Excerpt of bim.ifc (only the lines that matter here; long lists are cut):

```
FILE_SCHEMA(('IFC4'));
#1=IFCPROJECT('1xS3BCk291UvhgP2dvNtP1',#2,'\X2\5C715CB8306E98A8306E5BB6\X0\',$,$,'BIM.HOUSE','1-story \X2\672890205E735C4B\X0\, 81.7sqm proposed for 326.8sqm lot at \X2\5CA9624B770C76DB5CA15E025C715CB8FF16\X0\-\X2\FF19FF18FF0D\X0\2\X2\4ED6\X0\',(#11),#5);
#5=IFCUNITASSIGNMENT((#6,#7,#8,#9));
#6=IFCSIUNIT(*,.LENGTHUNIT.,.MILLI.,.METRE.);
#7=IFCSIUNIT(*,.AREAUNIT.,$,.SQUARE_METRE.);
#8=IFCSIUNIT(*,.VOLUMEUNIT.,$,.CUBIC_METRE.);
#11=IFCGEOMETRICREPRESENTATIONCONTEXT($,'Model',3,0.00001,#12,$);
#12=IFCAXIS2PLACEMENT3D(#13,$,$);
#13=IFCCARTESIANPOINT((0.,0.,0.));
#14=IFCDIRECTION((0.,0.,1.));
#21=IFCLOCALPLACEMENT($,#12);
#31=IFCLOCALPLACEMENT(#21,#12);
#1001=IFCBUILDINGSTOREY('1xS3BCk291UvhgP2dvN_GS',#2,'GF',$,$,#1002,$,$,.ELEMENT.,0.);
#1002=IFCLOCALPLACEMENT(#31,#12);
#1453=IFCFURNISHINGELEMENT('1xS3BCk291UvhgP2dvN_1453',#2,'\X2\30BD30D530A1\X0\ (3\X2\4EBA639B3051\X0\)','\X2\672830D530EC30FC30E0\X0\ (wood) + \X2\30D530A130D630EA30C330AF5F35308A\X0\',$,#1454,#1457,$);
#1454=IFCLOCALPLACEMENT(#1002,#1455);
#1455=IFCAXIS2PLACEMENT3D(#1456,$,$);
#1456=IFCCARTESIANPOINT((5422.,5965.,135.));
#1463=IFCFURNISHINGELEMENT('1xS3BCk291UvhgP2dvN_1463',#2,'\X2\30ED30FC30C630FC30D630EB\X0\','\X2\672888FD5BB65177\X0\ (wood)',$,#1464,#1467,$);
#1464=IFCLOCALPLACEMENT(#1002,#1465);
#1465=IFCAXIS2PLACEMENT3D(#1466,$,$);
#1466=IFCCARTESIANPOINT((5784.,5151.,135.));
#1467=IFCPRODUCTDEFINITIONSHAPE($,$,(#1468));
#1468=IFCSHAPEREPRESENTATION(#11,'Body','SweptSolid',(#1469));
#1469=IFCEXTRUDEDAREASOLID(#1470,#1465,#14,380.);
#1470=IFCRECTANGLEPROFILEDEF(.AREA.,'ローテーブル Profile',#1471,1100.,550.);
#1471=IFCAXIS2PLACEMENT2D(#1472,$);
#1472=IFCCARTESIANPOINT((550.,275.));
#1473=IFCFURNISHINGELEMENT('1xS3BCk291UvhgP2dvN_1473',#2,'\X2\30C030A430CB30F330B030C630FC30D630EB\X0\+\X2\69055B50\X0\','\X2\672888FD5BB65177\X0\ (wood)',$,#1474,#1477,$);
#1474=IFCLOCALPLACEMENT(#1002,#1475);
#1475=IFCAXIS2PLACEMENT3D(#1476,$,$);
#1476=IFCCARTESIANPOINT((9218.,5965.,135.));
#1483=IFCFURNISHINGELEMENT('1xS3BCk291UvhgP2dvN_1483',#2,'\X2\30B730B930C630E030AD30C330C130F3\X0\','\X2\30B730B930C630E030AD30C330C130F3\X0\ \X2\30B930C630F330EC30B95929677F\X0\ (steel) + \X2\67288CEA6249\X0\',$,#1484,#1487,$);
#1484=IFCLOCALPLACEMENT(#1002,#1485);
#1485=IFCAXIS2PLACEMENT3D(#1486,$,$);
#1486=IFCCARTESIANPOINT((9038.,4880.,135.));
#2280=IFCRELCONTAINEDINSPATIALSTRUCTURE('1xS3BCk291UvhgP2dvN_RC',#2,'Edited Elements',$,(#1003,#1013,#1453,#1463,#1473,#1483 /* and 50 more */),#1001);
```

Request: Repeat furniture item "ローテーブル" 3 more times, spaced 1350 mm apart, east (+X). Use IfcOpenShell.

```python
import numpy as np
import ifcopenshell
import ifcopenshell.api.geometry
import ifcopenshell.api.root
import ifcopenshell.util.element
import ifcopenshell.util.placement
import ifcopenshell.util.unit

model = ifcopenshell.open("bim.ifc")
unit_scale = ifcopenshell.util.unit.calculate_unit_scale(model)


def reuse_history(source, copy):
    """copy_class also copies each property set's owner history, people and application; keep the originals."""
    for rel in copy.IsDefinedBy:
        if rel.is_a("IfcRelDefinesByProperties") and (history := rel.RelatingPropertyDefinition.OwnerHistory):
            rel.RelatingPropertyDefinition.OwnerHistory = source.OwnerHistory
            ifcopenshell.util.element.remove_deep2(model, history)


source = model.by_id(1463)
base = ifcopenshell.util.placement.get_local_placement(source.ObjectPlacement)
step = np.array([1.0, 0.0, 0.0]) * 1.35 / unit_scale

for i in range(1, 4):
    copy = ifcopenshell.api.root.copy_class(model, product=source)
    copy.Representation = ifcopenshell.util.element.copy_deep(
        model, source.Representation, exclude=["IfcGeometricRepresentationContext", "IfcRepresentationMap"]
    )
    reuse_history(source, copy)
    matrix = base.copy()
    matrix[:3, 3] += i * step
    print("added at", matrix[:3, 3].round(3) + 0.0)
    ifcopenshell.api.geometry.edit_object_placement(model, product=copy, matrix=matrix, is_si=False)

model.write("bim_rev.ifc")
```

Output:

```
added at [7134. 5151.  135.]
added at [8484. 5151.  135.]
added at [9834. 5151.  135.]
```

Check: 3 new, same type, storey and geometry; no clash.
